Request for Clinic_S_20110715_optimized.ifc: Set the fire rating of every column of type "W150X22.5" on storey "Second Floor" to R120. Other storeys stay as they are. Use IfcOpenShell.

First a look at what the model holds.

```python
import ifcopenshell
import ifcopenshell.util.element

model = ifcopenshell.open("Clinic_S_20110715_optimized.ifc")
print(model.schema)
storey = next(s for s in model.by_type("IfcBuildingStorey") if s.Name == "Second Floor")
columns = [e for e in ifcopenshell.util.element.get_decomposition(storey) if e.is_a("IfcColumn")]
seen = {}
for e in columns:
    element_type = ifcopenshell.util.element.get_type(e)
    key = (element_type.Name if element_type != e and element_type else None, ifcopenshell.util.element.get_pset(e, "Pset_ColumnCommon", "FireRating"))
    seen[key] = seen.get(key, 0) + 1
for (name, value), count in sorted(seen.items(), key=str):
    print(count, "x", name, "|", value)
```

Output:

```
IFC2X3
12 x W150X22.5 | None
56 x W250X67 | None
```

```python
import ifcopenshell
import ifcopenshell.api.pset
import ifcopenshell.util.element

model = ifcopenshell.open("Clinic_S_20110715_optimized.ifc")

storey = next(s for s in model.by_type("IfcBuildingStorey") if s.Name == "Second Floor")
columns = [e for e in ifcopenshell.util.element.get_decomposition(storey) if e.is_a("IfcColumn")]

count = 0
for e in columns:
    element_type = ifcopenshell.util.element.get_type(e)
    if element_type in (None, e) or element_type.Name != "W150X22.5":
        continue
    # add_pset returns the element's existing set when there is one.
    pset = ifcopenshell.api.pset.add_pset(model, product=e, name="Pset_ColumnCommon")
    ifcopenshell.api.pset.edit_pset(model, pset=pset, properties={"FireRating": "R120"})
    count += 1

print(count, "columns updated")

model.write("Clinic_S_20110715_optimized_updated.ifc")
```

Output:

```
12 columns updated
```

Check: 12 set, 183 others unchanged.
